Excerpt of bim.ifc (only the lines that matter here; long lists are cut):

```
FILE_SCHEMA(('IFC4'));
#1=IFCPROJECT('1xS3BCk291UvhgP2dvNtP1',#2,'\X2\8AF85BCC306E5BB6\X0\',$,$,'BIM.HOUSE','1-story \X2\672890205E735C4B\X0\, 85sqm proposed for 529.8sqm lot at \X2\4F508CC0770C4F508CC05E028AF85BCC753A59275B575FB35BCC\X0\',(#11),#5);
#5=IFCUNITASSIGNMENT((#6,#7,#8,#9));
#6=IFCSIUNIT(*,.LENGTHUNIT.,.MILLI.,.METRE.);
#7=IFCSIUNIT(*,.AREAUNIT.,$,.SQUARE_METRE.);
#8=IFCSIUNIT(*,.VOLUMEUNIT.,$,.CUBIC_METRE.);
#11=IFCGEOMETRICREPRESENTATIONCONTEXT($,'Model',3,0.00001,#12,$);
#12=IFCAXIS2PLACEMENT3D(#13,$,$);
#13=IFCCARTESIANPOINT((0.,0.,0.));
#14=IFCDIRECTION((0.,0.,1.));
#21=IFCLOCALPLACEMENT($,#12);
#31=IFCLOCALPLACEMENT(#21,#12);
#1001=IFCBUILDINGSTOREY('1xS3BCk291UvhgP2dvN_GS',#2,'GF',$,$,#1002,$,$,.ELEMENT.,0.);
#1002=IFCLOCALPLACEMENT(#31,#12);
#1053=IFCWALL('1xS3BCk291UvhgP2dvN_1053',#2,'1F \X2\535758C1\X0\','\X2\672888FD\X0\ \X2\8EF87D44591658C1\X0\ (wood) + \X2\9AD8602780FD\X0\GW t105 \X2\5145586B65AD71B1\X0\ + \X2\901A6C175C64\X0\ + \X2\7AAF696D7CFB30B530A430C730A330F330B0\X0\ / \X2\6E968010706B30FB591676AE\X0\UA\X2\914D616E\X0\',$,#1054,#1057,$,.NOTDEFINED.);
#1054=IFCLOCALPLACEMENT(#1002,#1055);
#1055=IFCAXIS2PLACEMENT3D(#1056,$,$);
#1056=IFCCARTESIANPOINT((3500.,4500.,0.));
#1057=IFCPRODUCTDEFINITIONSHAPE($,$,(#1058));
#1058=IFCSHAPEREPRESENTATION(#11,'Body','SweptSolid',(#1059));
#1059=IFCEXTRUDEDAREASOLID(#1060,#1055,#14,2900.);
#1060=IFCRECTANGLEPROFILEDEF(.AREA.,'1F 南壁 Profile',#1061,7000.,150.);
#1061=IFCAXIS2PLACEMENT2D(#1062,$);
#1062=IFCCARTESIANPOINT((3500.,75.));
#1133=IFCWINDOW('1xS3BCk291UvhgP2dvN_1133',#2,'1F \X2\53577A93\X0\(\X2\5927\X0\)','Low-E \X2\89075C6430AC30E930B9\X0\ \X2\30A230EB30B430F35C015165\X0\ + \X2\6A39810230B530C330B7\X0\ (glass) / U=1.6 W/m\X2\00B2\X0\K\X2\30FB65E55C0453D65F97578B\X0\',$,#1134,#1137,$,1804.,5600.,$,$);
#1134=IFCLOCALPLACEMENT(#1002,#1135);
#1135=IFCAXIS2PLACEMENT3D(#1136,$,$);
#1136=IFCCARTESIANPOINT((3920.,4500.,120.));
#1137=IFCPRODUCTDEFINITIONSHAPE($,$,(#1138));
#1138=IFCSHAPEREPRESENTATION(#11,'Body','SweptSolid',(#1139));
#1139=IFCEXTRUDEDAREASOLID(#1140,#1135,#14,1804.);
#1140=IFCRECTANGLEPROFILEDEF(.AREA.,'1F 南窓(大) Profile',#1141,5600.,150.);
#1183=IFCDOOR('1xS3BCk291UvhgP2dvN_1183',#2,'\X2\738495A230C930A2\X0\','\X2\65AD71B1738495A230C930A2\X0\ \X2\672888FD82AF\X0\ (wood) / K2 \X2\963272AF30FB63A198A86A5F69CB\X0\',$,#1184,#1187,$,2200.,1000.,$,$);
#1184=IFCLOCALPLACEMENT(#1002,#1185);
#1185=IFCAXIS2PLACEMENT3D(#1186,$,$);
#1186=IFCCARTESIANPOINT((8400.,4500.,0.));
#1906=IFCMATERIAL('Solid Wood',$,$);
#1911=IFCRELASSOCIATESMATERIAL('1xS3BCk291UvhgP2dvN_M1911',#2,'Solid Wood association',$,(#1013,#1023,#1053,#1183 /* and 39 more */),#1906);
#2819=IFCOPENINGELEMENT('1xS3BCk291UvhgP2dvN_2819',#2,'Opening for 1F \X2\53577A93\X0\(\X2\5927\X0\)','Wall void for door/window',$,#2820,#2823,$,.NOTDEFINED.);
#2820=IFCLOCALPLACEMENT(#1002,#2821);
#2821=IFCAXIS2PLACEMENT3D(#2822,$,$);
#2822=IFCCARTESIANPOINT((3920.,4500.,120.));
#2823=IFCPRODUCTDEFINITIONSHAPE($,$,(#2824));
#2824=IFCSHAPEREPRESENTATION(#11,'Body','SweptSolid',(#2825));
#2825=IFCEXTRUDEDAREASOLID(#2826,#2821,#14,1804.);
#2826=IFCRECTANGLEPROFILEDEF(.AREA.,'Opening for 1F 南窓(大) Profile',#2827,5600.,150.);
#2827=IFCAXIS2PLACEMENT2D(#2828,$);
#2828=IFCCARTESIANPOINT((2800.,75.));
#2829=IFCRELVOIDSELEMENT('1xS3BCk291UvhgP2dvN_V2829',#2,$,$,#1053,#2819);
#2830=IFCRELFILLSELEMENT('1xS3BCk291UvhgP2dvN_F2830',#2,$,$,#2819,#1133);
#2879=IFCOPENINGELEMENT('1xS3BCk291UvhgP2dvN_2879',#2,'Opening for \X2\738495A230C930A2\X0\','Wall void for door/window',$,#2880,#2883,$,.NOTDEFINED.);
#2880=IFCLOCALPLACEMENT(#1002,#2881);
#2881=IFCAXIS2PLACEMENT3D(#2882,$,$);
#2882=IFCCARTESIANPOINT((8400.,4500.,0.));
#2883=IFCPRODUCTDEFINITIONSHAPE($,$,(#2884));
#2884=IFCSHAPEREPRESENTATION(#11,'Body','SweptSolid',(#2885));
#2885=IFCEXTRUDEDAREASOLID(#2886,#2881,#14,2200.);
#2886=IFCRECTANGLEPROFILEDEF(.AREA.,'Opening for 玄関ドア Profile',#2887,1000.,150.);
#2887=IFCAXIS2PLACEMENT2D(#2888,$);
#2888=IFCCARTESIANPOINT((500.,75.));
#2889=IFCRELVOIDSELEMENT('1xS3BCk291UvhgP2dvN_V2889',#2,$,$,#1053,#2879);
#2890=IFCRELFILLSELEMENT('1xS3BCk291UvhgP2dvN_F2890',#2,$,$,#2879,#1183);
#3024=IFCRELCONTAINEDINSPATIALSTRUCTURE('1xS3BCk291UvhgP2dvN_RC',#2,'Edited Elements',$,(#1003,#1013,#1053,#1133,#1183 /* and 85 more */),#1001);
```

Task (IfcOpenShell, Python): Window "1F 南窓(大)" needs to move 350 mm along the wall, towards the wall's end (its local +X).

```python
import ifcopenshell
import ifcopenshell.api.geometry
import ifcopenshell.util.placement

model = ifcopenshell.open("bim.ifc")

window = model.by_id(1133)
opening = window.FillsVoids[0].RelatingOpeningElement
wall = opening.VoidsElements[0].RelatingBuildingElement

wall_matrix = ifcopenshell.util.placement.get_local_placement(wall.ObjectPlacement)
shift = wall_matrix[:3, 0] * 350.0
before = ifcopenshell.util.placement.get_local_placement(window.ObjectPlacement)[:3, 3].copy()

# The window is not placed relative to its opening, so move both.
for product in (opening, window):
    matrix = ifcopenshell.util.placement.get_local_placement(product.ObjectPlacement)
    matrix[:3, 3] += shift
    ifcopenshell.api.geometry.edit_object_placement(model, product=product, matrix=matrix, is_si=False)

after = ifcopenshell.util.placement.get_local_placement(window.ObjectPlacement)[:3, 3]
print("window moved by", (after - before).round(3) + 0.0)

model.write("bim-out.ifc")
```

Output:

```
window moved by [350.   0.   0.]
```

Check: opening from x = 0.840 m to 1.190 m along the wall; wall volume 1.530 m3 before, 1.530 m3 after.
